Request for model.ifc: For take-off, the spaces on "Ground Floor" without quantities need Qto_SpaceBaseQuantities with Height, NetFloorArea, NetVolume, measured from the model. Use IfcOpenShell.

First a look at what the model holds.

```python
import ifcopenshell
import ifcopenshell.util.element
import ifcopenshell.util.unit

model = ifcopenshell.open("model.ifc")
print(model.schema)
for unit_type in ("LENGTHUNIT", "AREAUNIT", "VOLUMEUNIT"):
    print(unit_type, ifcopenshell.util.unit.calculate_unit_scale(model, unit_type))
storey = next(s for s in model.by_type("IfcBuildingStorey") if s.Name == "Ground Floor")
spaces = [e for e in ifcopenshell.util.element.get_decomposition(storey) if e.is_a("IfcSpace")]
for e in sorted(spaces, key=lambda e: e.id()):
    print(e.id(), e.is_a(), e.Name, list(ifcopenshell.util.element.get_psets(e, qtos_only=True)), sep=" | ")
```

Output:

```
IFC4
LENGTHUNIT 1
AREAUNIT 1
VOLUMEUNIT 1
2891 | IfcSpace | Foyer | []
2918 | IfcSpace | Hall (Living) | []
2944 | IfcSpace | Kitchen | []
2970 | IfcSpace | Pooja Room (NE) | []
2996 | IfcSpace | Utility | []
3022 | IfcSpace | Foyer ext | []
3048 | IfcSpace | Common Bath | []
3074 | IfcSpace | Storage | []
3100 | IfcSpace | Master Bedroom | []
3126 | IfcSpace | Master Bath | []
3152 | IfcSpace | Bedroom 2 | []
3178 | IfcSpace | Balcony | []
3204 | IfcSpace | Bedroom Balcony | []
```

```python
import ifcopenshell
import ifcopenshell.api.pset
import ifcopenshell.geom
import ifcopenshell.util.element
import ifcopenshell.util.shape
import ifcopenshell.util.unit

model = ifcopenshell.open("model.ifc")
unit_scale = ifcopenshell.util.unit.calculate_unit_scale(model)
area_scale = ifcopenshell.util.unit.calculate_unit_scale(model, "AREAUNIT")
volume_scale = ifcopenshell.util.unit.calculate_unit_scale(model, "VOLUMEUNIT")
settings = ifcopenshell.geom.settings()

storey = next(s for s in model.by_type("IfcBuildingStorey") if s.Name == "Ground Floor")
spaces = [e for e in ifcopenshell.util.element.get_decomposition(storey) if e.is_a("IfcSpace")]

for e in sorted(spaces, key=lambda e: e.id()):
    if ifcopenshell.util.element.get_psets(e, qtos_only=True, should_inherit=False):
        continue
    # Geometry comes back in metres, in the element's own axes.
    shape = ifcopenshell.geom.create_shape(settings, e)
    values = {
        "Height": ifcopenshell.util.shape.get_z(shape.geometry) / unit_scale,
        "NetFloorArea": ifcopenshell.util.shape.get_footprint_area(shape.geometry) / area_scale,
        "NetVolume": ifcopenshell.util.shape.get_volume(shape.geometry) / volume_scale,
    }
    qto = ifcopenshell.api.pset.add_qto(model, product=e, name="Qto_SpaceBaseQuantities")
    ifcopenshell.api.pset.edit_qto(model, qto=qto, properties=values)
    print(e.id(), {k: round(v, 3) for k, v in values.items()})

model.write("model-out.ifc")
```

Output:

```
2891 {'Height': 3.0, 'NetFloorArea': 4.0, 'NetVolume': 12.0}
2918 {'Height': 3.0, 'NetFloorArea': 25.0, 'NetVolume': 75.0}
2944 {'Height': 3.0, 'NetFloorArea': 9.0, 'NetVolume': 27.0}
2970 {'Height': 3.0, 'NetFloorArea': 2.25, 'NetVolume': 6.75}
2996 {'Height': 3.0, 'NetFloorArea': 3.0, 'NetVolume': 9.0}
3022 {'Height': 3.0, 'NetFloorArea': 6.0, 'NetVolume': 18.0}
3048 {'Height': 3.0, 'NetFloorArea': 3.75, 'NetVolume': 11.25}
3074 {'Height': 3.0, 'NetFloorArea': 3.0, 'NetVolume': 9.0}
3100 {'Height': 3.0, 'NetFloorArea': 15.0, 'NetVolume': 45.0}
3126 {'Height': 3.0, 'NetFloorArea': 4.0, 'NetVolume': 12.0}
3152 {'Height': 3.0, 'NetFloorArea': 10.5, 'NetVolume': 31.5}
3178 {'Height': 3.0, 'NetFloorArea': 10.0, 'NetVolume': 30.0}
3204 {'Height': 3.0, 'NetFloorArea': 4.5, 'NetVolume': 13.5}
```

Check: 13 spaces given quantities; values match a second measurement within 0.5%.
